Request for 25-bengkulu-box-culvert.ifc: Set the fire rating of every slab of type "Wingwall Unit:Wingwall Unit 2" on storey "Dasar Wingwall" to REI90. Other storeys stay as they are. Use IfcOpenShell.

First a look at what the model holds.

```python
import ifcopenshell
import ifcopenshell.util.element

model = ifcopenshell.open("25-bengkulu-box-culvert.ifc")
print(model.schema)
storey = next(s for s in model.by_type("IfcBuildingStorey") if s.Name == "Dasar Wingwall")
slabs = [e for e in ifcopenshell.util.element.get_decomposition(storey) if e.is_a("IfcSlab")]
seen = {}
for e in slabs:
    element_type = ifcopenshell.util.element.get_type(e)
    key = (element_type.Name if element_type != e and element_type else None, ifcopenshell.util.element.get_pset(e, "Pset_SlabCommon", "FireRating"))
    seen[key] = seen.get(key, 0) + 1
for (name, value), count in sorted(seen.items(), key=str):
    print(count, "x", name, "|", value)
```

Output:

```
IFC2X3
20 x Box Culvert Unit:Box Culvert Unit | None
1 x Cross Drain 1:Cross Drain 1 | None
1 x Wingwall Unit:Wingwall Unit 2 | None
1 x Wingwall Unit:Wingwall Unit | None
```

```python
import ifcopenshell
import ifcopenshell.api.pset
import ifcopenshell.util.element

model = ifcopenshell.open("25-bengkulu-box-culvert.ifc")

storey = next(s for s in model.by_type("IfcBuildingStorey") if s.Name == "Dasar Wingwall")
slabs = [e for e in ifcopenshell.util.element.get_decomposition(storey) if e.is_a("IfcSlab")]

count = 0
for e in slabs:
    element_type = ifcopenshell.util.element.get_type(e)
    if element_type in (None, e) or element_type.Name != "Wingwall Unit:Wingwall Unit 2":
        continue
    # add_pset returns the element's existing set when there is one.
    pset = ifcopenshell.api.pset.add_pset(model, product=e, name="Pset_SlabCommon")
    ifcopenshell.api.pset.edit_pset(model, pset=pset, properties={"FireRating": "REI90"})
    count += 1

print(count, "slabs updated")

model.write("25-bengkulu-box-culvert-out.ifc")
```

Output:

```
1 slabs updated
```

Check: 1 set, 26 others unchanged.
